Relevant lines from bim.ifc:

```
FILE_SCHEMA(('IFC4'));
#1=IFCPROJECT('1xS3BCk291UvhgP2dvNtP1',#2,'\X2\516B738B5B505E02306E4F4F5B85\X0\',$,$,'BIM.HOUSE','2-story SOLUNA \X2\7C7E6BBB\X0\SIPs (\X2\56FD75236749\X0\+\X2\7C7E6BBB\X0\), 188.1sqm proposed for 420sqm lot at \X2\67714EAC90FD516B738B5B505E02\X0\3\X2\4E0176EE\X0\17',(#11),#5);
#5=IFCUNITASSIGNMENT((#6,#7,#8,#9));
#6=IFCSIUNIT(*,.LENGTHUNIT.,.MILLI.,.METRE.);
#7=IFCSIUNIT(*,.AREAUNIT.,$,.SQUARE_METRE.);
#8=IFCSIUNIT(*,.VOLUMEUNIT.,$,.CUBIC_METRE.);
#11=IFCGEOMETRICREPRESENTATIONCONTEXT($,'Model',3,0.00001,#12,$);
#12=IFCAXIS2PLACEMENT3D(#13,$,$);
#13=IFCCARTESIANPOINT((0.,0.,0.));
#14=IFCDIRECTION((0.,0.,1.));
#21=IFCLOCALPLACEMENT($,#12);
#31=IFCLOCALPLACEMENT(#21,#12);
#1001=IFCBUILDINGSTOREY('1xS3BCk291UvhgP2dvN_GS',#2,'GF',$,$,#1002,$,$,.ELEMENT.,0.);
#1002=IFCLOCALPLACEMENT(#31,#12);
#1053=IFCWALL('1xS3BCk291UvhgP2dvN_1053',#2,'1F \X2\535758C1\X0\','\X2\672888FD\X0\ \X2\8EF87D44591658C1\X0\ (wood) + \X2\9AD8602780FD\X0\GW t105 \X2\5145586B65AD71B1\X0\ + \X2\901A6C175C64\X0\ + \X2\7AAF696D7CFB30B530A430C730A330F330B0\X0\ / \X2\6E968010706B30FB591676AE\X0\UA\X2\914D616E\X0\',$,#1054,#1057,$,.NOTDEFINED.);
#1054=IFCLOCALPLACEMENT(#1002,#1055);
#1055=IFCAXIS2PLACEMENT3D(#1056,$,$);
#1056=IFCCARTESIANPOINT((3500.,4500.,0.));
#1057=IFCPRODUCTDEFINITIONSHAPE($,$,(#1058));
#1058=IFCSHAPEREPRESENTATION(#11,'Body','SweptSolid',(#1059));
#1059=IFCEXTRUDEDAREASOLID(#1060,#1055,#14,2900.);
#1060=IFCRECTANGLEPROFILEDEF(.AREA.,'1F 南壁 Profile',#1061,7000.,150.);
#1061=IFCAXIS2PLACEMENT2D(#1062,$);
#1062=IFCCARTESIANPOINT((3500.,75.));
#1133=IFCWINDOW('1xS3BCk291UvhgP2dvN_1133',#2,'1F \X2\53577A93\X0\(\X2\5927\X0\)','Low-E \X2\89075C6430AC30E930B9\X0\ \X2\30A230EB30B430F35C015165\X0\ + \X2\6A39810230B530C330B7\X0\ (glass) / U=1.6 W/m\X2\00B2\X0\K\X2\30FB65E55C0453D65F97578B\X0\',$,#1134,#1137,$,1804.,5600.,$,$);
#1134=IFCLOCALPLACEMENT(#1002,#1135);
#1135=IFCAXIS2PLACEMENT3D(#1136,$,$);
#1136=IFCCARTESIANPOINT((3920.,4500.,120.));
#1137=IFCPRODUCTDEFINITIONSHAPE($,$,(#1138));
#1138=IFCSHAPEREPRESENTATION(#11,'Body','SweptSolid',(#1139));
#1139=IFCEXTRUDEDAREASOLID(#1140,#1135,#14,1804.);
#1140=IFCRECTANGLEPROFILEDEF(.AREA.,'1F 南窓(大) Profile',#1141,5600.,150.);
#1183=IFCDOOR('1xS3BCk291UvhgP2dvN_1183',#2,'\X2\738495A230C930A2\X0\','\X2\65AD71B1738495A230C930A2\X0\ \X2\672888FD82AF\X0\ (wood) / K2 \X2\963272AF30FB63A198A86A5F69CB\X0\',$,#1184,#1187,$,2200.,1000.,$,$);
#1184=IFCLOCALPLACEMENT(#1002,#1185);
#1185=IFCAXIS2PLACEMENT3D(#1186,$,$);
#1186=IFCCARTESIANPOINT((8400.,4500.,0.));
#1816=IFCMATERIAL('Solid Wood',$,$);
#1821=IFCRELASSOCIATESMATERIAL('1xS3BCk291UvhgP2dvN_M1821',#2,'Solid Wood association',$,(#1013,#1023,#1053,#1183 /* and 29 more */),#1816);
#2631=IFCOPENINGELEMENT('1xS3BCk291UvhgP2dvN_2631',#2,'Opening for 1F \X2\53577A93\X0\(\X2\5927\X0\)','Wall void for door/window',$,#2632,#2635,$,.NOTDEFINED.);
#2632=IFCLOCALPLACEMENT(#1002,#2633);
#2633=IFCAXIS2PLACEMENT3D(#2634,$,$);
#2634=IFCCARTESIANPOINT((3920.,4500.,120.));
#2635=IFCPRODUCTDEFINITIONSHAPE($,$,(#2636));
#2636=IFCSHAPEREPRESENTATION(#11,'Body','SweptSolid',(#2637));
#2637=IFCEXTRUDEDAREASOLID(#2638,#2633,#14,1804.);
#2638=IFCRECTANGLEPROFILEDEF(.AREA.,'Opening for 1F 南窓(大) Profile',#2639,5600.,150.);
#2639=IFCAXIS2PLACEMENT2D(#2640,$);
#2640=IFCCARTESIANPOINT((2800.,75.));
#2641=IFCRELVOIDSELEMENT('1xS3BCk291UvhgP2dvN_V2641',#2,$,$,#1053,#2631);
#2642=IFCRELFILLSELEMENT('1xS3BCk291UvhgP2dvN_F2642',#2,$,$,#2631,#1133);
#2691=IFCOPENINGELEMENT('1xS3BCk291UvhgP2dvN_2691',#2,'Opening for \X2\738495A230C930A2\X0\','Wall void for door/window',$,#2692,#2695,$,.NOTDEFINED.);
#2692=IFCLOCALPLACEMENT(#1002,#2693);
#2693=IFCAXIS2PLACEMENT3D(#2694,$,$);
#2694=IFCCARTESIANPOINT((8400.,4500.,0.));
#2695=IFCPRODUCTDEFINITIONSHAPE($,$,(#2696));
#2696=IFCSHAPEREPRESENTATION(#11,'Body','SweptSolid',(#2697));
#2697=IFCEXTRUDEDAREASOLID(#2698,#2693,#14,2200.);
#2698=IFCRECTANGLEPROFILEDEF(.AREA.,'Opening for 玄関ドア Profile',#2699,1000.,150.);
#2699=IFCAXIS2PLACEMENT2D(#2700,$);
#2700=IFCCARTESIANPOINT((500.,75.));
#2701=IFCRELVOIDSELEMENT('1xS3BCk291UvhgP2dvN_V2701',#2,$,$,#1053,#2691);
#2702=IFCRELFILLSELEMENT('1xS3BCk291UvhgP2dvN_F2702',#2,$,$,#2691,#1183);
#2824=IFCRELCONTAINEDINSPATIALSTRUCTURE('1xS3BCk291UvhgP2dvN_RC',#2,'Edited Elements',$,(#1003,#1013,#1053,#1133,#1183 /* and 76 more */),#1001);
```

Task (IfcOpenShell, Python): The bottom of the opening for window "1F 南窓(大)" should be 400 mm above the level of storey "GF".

```python
import numpy as np
import ifcopenshell
import ifcopenshell.api.geometry
import ifcopenshell.geom
import ifcopenshell.util.element
import ifcopenshell.util.placement
import ifcopenshell.util.shape
import ifcopenshell.util.unit

model = ifcopenshell.open("bim.ifc")
unit_scale = ifcopenshell.util.unit.calculate_unit_scale(model)

window = model.by_id(1133)
opening = window.FillsVoids[0].RelatingOpeningElement
storey = ifcopenshell.util.element.get_container(window, ifc_class="IfcBuildingStorey")
level = ifcopenshell.util.placement.get_local_placement(storey.ObjectPlacement)[2, 3]

# The opening's origin need not be at the sill, so measure its lowest point.
shape = ifcopenshell.geom.create_shape(ifcopenshell.geom.settings(), opening)
bottom = ifcopenshell.util.shape.get_shape_bottom_elevation(shape, shape.geometry) / unit_scale
dz = level + 0.4 / unit_scale - bottom

shift = np.array([0.0, 0.0, dz])
# The window is not placed relative to its opening, so move both.
for product in (opening, window):
    matrix = ifcopenshell.util.placement.get_local_placement(product.ObjectPlacement)
    matrix[:3, 3] += shift
    ifcopenshell.api.geometry.edit_object_placement(model, product=product, matrix=matrix, is_si=False)

print(f"moved by {dz * unit_scale:+.3f} m")

model.write("bim_v2.ifc")
```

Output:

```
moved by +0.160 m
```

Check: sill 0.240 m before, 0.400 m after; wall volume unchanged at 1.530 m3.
